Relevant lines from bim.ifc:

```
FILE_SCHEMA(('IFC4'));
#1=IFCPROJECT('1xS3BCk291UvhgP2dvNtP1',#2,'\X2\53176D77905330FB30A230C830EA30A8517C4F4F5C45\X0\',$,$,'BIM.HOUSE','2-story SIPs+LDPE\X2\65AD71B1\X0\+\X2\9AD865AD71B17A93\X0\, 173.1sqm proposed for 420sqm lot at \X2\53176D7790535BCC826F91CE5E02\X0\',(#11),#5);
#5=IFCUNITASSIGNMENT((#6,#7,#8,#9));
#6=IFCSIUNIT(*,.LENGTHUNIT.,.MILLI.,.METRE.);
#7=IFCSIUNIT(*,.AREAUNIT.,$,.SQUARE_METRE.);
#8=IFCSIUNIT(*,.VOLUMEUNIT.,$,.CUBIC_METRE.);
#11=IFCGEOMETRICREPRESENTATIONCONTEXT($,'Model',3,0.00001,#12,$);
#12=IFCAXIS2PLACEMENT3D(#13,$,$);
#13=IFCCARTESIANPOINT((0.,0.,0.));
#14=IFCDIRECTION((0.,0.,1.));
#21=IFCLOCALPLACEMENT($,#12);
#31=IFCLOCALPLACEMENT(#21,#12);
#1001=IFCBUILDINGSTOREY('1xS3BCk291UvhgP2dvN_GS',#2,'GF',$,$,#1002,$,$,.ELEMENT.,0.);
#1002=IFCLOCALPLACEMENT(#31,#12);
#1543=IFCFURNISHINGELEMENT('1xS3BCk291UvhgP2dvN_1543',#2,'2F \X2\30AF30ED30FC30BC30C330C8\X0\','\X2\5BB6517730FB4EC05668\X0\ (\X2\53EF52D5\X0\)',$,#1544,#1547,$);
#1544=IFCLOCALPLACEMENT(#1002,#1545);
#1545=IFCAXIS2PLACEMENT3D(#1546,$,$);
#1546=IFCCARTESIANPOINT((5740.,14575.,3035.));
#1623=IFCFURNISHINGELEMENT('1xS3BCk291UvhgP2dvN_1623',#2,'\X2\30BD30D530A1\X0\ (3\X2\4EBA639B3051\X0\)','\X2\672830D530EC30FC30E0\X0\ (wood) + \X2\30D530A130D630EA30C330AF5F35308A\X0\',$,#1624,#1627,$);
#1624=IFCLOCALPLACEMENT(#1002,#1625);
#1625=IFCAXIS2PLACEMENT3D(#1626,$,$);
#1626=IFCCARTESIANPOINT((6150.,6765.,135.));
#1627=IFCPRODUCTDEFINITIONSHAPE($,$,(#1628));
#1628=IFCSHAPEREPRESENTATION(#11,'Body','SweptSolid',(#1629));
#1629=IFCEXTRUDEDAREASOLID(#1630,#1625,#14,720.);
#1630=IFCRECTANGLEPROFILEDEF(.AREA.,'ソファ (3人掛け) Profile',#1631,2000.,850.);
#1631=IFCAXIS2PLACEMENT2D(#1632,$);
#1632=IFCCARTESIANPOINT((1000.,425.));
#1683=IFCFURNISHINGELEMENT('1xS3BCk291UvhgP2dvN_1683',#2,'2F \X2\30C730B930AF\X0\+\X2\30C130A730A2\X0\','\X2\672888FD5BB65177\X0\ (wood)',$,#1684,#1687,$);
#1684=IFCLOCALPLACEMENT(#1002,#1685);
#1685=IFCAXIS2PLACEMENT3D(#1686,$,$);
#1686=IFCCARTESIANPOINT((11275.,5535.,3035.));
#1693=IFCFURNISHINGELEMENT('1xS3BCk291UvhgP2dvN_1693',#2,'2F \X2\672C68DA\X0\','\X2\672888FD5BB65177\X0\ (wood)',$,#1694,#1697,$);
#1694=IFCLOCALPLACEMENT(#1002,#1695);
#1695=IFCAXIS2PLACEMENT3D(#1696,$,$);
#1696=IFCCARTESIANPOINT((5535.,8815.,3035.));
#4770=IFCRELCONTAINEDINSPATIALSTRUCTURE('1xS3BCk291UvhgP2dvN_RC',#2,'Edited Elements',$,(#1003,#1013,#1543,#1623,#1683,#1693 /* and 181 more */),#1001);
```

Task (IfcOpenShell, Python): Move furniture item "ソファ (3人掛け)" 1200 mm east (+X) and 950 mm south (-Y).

```python
import ifcopenshell
import ifcopenshell.api.geometry
import ifcopenshell.util.placement
import ifcopenshell.util.unit

model = ifcopenshell.open("bim.ifc")
unit_scale = ifcopenshell.util.unit.calculate_unit_scale(model)

item = model.by_id(1623)
matrix = ifcopenshell.util.placement.get_local_placement(item.ObjectPlacement)
matrix[0, 3] += 1.2 / unit_scale
matrix[1, 3] -= 0.95 / unit_scale
ifcopenshell.api.geometry.edit_object_placement(model, product=item, matrix=matrix, is_si=False)

print(ifcopenshell.util.placement.get_local_placement(item.ObjectPlacement).round(3) + 0.0)

model.write("bim-out.ifc")
```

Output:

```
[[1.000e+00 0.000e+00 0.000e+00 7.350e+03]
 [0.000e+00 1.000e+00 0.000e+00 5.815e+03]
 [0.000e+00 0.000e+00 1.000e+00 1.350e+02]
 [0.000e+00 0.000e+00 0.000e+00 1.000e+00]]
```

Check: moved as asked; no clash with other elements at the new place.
